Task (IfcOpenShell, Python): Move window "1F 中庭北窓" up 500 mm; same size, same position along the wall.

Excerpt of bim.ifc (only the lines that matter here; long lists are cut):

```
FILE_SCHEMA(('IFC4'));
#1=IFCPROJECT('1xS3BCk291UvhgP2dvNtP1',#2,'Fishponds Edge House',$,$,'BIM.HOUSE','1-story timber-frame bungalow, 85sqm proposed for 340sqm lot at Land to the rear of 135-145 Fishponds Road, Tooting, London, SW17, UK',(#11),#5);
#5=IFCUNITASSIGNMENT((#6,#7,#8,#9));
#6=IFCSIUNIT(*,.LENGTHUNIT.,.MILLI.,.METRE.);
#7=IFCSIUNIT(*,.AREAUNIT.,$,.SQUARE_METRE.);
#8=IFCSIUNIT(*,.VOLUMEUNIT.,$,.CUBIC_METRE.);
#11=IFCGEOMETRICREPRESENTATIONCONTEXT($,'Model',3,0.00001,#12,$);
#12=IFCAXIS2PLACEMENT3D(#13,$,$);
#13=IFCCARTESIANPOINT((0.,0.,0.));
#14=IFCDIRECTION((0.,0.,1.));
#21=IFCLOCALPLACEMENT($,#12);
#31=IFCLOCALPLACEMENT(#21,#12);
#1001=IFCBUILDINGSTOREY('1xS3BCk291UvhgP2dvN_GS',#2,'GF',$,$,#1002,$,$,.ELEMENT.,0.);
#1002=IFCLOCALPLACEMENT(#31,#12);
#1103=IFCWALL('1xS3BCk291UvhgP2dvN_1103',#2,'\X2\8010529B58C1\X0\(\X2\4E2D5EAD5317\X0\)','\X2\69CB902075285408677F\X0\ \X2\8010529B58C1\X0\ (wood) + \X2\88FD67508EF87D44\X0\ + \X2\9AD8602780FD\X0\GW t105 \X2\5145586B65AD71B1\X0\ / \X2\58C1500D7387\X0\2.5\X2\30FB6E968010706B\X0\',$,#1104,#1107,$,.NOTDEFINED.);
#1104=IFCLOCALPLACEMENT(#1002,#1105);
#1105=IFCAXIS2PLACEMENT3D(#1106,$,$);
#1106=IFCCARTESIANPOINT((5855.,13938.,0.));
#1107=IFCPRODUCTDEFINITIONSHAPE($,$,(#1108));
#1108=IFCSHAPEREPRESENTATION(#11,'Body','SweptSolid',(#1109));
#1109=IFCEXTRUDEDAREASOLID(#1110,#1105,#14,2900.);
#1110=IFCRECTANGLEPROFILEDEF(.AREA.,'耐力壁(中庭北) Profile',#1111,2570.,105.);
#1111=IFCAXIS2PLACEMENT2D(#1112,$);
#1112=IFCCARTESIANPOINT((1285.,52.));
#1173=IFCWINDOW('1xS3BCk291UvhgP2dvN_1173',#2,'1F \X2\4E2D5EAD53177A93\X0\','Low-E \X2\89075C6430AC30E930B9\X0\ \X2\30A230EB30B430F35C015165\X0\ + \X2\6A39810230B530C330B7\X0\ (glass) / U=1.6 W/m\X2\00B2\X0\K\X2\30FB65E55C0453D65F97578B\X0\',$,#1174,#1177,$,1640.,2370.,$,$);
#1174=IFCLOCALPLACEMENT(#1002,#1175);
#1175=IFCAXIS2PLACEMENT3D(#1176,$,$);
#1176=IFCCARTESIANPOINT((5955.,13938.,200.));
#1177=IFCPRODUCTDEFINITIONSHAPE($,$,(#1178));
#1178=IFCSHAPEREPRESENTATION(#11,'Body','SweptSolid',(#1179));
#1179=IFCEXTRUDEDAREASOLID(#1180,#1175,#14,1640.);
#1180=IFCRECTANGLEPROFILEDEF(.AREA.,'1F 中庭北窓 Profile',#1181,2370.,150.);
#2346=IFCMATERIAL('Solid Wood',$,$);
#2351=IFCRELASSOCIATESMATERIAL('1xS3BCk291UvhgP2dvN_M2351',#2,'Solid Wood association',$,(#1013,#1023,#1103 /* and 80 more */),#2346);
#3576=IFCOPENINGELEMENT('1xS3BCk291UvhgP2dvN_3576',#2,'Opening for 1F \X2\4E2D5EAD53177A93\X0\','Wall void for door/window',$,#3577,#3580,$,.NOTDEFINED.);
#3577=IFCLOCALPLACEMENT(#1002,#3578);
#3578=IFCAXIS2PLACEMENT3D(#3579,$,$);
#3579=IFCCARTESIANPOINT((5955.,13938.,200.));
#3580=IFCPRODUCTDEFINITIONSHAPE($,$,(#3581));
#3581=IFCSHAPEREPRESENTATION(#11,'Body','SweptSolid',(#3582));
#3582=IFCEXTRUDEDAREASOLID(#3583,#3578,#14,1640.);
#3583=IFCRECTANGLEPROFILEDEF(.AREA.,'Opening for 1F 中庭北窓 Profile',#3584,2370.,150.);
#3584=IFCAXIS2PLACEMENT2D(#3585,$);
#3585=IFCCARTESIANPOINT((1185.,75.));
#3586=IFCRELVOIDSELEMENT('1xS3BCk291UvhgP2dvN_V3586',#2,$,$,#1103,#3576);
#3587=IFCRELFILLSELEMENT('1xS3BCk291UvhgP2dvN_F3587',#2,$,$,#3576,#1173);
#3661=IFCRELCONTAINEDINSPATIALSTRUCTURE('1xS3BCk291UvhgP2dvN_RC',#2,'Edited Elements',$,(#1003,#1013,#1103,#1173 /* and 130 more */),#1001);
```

```python
import numpy as np
import ifcopenshell
import ifcopenshell.api.geometry
import ifcopenshell.util.placement
import ifcopenshell.util.unit

model = ifcopenshell.open("bim.ifc")
unit_scale = ifcopenshell.util.unit.calculate_unit_scale(model)

window = model.by_id(1173)
opening = window.FillsVoids[0].RelatingOpeningElement
dz = 0.5 / unit_scale

shift = np.array([0.0, 0.0, dz])
# The window is not placed relative to its opening, so move both.
for product in (opening, window):
    matrix = ifcopenshell.util.placement.get_local_placement(product.ObjectPlacement)
    matrix[:3, 3] += shift
    ifcopenshell.api.geometry.edit_object_placement(model, product=product, matrix=matrix, is_si=False)

print(f"moved by {dz * unit_scale:+.3f} m")

model.write("bim_edited.ifc")
```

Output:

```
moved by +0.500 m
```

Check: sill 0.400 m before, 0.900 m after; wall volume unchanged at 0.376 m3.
